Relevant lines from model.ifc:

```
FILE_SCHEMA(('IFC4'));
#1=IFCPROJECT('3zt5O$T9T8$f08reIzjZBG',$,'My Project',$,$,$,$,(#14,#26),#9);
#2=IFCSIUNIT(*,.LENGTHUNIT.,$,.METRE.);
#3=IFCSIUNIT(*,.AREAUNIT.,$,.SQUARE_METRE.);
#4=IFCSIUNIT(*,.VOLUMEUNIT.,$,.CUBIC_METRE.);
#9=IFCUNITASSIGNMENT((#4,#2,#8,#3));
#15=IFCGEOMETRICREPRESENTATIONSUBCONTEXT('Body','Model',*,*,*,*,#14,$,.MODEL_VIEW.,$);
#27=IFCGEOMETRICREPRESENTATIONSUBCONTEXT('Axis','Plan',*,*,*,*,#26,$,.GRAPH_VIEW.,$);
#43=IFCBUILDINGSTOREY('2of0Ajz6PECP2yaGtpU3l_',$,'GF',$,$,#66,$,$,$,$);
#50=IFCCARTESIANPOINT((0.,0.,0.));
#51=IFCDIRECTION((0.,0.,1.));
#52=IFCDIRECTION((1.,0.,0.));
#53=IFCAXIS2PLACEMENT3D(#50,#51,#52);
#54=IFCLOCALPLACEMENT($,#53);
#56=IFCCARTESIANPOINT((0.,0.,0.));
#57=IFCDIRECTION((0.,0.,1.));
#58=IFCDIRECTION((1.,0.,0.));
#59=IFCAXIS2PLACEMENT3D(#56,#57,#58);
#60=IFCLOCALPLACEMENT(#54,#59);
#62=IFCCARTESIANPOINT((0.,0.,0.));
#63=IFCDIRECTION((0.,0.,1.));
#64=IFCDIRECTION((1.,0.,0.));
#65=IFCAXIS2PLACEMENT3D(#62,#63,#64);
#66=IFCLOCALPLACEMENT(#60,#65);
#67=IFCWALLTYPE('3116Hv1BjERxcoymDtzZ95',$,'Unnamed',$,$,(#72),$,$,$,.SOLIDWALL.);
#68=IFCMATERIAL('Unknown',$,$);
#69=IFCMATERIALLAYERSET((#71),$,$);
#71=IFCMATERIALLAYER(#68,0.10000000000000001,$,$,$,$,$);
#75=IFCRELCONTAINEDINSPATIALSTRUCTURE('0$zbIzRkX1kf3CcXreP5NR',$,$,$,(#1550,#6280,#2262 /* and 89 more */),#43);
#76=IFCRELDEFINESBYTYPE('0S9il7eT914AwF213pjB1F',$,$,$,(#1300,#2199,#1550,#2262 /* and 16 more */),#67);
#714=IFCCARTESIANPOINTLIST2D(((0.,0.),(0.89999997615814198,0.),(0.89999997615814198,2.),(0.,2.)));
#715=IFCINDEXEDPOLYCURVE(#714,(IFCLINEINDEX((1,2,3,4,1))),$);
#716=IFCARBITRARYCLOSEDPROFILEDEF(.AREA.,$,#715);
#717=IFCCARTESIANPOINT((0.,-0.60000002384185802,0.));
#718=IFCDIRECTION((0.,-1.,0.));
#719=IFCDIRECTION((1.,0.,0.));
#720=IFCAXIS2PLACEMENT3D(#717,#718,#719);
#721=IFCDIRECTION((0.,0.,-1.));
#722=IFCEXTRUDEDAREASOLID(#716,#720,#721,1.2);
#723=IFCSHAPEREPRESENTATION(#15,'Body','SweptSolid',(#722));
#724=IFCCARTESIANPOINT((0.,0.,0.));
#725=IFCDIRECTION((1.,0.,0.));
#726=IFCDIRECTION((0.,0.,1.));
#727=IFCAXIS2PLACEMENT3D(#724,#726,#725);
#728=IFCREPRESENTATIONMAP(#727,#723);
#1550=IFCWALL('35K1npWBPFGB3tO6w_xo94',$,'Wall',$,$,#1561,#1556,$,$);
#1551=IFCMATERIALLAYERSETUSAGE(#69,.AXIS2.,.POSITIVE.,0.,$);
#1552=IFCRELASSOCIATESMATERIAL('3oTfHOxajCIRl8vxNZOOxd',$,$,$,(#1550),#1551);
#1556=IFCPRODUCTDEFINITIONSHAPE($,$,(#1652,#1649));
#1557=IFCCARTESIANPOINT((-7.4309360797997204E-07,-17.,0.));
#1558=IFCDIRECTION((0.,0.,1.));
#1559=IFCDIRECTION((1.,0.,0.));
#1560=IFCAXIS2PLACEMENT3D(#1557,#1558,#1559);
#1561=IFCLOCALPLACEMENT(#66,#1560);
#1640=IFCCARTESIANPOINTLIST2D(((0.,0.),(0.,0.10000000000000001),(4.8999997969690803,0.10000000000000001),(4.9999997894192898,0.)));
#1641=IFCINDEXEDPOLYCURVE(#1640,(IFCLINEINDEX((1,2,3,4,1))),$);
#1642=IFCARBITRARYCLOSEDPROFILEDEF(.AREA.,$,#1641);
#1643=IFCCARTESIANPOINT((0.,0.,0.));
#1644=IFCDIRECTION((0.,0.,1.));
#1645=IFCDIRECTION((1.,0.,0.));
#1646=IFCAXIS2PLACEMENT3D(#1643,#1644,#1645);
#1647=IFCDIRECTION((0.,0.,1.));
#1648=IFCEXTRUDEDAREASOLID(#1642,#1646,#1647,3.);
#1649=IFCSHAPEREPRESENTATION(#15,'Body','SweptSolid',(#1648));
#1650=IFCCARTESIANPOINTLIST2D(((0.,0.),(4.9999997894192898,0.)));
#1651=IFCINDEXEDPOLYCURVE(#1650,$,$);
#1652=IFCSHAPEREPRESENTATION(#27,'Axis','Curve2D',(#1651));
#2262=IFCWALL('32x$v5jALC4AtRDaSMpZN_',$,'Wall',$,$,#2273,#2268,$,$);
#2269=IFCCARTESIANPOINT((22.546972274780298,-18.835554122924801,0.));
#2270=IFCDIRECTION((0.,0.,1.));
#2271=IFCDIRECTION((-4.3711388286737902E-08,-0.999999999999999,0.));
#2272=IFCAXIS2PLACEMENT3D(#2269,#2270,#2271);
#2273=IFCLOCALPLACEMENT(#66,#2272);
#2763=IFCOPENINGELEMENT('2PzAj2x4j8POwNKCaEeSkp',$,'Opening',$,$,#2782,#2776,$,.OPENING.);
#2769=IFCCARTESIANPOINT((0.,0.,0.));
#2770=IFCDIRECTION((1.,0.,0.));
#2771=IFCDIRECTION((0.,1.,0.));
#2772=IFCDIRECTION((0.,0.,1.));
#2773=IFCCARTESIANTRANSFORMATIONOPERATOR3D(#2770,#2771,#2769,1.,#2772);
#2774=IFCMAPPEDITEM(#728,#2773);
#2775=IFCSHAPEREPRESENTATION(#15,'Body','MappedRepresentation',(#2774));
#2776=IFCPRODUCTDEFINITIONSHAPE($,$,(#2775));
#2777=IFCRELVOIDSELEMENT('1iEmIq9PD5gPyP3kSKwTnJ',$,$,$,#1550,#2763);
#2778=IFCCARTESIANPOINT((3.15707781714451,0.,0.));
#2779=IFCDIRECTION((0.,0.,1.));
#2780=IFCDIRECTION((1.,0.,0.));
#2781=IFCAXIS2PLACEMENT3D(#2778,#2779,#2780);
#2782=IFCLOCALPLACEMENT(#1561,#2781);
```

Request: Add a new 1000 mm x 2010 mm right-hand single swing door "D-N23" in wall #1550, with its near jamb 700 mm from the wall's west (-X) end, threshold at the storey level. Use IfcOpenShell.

```python
import numpy as np
import ifcopenshell
import ifcopenshell.api.feature
import ifcopenshell.api.geometry
import ifcopenshell.api.root
import ifcopenshell.api.spatial
import ifcopenshell.geom
import ifcopenshell.util.element
import ifcopenshell.util.placement
import ifcopenshell.util.representation
import ifcopenshell.util.shape
import ifcopenshell.util.unit

model = ifcopenshell.open("model.ifc")
unit_scale = ifcopenshell.util.unit.calculate_unit_scale(model)
settings = ifcopenshell.geom.settings()


def volume(element):
    """Net volume in cubic metres, openings subtracted."""
    shape = ifcopenshell.geom.create_shape(settings, element)
    return ifcopenshell.util.shape.get_volume(shape.geometry)


wall = model.by_guid("35K1npWBPFGB3tO6w_xo94")
storey = ifcopenshell.util.element.get_container(wall, ifc_class="IfcBuildingStorey")
context = ifcopenshell.util.representation.get_context(model, "Model", "Body", "MODEL_VIEW")
before = volume(wall)

width, height, from_end, sill = 1, 2.01, 0.7, 0.0  # metres

# The wall runs along its own X axis, and the end named is its -X end.
wall_shape = ifcopenshell.geom.create_shape(settings, wall)
x, y, z = ifcopenshell.util.shape.get_vertices(wall_shape.geometry).T
start = x.min() + from_end
face, thickness = float(y.min()), float(y.max() - y.min())
wall_matrix = ifcopenshell.util.placement.get_local_placement(wall.ObjectPlacement)
level = ifcopenshell.util.placement.get_local_placement(storey.ObjectPlacement)[2, 3]


def in_wall(x, y):
    """Placement at x, y metres in the wall's axes, at sill height."""
    matrix = wall_matrix.copy()
    matrix[:, 3] = wall_matrix @ np.array([x / unit_scale, y / unit_scale, 0.0, 1.0])
    matrix[2, 3] = level + sill / unit_scale
    return matrix


# Opening: a box that overshoots both wall faces by 50 mm.
opening = ifcopenshell.api.root.create_entity(model, ifc_class="IfcOpeningElement", predefined_type="OPENING")
box = ifcopenshell.api.geometry.add_wall_representation(
    model, context=context, length=width, height=height, thickness=thickness + 0.1
)
ifcopenshell.api.geometry.assign_representation(model, product=opening, representation=box)
ifcopenshell.api.geometry.edit_object_placement(model, product=opening, matrix=in_wall(start, face - 0.05), is_si=False)
ifcopenshell.api.feature.add_feature(model, feature=opening, element=wall)

door = ifcopenshell.api.root.create_entity(model, ifc_class="IfcDoor", name="D-N23", predefined_type="DOOR")
door.OverallWidth, door.OverallHeight = width / unit_scale, height / unit_scale
door.OperationType = "SINGLE_SWING_RIGHT"
body = ifcopenshell.api.geometry.add_door_representation(
    model,
    context=context,
    overall_width=door.OverallWidth,
    overall_height=door.OverallHeight,
    operation_type="SINGLE_SWING_RIGHT",
    lining_properties={"LiningDepth": thickness / unit_scale, "ThresholdDepth": thickness / unit_scale},
)
ifcopenshell.api.geometry.assign_representation(model, product=door, representation=body)
ifcopenshell.api.spatial.assign_container(model, products=[door], relating_structure=storey)
ifcopenshell.api.feature.add_filling(model, opening=opening, element=door)

# The lining spans the wall, so the door starts at the wall face.
ifcopenshell.api.geometry.edit_object_placement(model, product=door, matrix=in_wall(start, face), is_si=False)

after = volume(wall)

print(f"wall volume {before:.3f} -> {after:.3f} m3")

model.write("model_edited.ifc")
```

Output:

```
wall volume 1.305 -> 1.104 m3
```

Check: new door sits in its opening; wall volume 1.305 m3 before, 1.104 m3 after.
